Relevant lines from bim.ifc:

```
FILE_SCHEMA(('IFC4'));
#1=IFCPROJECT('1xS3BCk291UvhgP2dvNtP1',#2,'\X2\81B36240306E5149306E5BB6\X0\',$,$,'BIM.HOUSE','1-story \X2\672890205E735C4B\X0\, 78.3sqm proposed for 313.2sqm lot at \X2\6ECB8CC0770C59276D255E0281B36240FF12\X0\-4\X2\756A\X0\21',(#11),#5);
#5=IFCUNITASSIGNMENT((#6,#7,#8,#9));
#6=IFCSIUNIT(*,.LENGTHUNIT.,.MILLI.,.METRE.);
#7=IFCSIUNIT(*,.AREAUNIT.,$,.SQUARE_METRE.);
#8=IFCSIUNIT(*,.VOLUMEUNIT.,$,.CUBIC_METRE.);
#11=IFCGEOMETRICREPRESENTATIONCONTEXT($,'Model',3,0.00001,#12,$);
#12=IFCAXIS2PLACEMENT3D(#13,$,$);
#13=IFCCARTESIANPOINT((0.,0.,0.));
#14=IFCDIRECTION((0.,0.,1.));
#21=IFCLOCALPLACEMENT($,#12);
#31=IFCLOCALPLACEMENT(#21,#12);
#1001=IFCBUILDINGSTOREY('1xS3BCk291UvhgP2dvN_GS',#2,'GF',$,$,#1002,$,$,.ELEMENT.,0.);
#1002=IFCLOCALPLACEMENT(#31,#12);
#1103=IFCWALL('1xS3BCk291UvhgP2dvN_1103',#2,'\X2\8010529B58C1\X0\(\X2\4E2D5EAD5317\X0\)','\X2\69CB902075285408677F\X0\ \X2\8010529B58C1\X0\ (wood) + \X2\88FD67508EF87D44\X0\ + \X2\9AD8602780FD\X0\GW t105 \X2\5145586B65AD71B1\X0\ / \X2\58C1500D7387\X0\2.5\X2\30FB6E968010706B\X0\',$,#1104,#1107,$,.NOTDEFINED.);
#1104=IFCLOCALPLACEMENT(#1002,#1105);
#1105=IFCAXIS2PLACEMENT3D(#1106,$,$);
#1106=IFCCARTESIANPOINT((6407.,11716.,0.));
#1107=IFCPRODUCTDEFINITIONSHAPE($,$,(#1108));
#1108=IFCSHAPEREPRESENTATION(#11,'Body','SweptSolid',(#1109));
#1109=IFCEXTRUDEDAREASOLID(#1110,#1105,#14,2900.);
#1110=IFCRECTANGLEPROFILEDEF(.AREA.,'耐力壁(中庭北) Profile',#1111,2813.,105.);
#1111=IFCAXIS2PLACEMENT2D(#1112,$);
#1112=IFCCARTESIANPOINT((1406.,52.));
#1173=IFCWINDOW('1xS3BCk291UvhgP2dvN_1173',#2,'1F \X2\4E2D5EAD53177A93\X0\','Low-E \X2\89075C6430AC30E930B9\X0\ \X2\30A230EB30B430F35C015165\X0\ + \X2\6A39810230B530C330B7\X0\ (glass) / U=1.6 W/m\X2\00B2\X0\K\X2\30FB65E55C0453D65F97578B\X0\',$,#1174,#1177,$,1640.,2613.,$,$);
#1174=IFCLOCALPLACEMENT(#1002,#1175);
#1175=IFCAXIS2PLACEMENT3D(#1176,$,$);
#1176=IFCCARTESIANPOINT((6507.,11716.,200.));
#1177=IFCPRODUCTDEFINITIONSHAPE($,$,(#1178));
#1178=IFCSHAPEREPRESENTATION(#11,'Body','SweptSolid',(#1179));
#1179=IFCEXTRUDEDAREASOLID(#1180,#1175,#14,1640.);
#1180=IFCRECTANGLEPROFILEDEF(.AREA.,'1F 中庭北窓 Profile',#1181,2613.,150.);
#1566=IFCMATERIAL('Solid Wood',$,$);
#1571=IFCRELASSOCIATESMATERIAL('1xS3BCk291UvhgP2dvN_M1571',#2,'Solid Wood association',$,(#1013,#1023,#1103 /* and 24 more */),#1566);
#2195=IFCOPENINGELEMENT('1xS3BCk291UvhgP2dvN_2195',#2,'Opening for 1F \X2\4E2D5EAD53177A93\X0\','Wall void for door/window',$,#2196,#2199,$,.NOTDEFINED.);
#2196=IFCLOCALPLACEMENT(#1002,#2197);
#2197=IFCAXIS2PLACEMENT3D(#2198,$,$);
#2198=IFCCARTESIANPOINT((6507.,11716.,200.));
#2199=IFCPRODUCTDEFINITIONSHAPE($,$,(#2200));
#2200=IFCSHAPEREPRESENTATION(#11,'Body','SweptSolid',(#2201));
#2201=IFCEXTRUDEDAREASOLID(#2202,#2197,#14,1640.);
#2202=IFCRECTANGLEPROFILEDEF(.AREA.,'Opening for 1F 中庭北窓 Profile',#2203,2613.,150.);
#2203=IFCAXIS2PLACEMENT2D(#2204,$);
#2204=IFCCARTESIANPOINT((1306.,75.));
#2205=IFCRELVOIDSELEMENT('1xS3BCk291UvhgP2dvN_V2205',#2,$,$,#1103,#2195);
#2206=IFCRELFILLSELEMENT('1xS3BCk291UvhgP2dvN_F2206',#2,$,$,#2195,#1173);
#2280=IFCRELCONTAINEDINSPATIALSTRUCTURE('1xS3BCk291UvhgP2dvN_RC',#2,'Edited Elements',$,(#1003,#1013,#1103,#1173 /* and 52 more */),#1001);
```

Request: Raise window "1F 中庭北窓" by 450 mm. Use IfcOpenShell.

```python
import numpy as np
import ifcopenshell
import ifcopenshell.api.geometry
import ifcopenshell.util.placement
import ifcopenshell.util.unit

model = ifcopenshell.open("bim.ifc")
unit_scale = ifcopenshell.util.unit.calculate_unit_scale(model)

window = model.by_guid("1xS3BCk291UvhgP2dvN_1173")
opening = window.FillsVoids[0].RelatingOpeningElement
dz = 0.45 / unit_scale

shift = np.array([0.0, 0.0, dz])
# The window is not placed relative to its opening, so move both.
for product in (opening, window):
    matrix = ifcopenshell.util.placement.get_local_placement(product.ObjectPlacement)
    matrix[:3, 3] += shift
    ifcopenshell.api.geometry.edit_object_placement(model, product=product, matrix=matrix, is_si=False)

print(f"moved by {dz * unit_scale:+.3f} m")

model.write("bim-out.ifc")
```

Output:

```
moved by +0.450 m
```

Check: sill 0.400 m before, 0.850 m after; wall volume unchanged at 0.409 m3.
